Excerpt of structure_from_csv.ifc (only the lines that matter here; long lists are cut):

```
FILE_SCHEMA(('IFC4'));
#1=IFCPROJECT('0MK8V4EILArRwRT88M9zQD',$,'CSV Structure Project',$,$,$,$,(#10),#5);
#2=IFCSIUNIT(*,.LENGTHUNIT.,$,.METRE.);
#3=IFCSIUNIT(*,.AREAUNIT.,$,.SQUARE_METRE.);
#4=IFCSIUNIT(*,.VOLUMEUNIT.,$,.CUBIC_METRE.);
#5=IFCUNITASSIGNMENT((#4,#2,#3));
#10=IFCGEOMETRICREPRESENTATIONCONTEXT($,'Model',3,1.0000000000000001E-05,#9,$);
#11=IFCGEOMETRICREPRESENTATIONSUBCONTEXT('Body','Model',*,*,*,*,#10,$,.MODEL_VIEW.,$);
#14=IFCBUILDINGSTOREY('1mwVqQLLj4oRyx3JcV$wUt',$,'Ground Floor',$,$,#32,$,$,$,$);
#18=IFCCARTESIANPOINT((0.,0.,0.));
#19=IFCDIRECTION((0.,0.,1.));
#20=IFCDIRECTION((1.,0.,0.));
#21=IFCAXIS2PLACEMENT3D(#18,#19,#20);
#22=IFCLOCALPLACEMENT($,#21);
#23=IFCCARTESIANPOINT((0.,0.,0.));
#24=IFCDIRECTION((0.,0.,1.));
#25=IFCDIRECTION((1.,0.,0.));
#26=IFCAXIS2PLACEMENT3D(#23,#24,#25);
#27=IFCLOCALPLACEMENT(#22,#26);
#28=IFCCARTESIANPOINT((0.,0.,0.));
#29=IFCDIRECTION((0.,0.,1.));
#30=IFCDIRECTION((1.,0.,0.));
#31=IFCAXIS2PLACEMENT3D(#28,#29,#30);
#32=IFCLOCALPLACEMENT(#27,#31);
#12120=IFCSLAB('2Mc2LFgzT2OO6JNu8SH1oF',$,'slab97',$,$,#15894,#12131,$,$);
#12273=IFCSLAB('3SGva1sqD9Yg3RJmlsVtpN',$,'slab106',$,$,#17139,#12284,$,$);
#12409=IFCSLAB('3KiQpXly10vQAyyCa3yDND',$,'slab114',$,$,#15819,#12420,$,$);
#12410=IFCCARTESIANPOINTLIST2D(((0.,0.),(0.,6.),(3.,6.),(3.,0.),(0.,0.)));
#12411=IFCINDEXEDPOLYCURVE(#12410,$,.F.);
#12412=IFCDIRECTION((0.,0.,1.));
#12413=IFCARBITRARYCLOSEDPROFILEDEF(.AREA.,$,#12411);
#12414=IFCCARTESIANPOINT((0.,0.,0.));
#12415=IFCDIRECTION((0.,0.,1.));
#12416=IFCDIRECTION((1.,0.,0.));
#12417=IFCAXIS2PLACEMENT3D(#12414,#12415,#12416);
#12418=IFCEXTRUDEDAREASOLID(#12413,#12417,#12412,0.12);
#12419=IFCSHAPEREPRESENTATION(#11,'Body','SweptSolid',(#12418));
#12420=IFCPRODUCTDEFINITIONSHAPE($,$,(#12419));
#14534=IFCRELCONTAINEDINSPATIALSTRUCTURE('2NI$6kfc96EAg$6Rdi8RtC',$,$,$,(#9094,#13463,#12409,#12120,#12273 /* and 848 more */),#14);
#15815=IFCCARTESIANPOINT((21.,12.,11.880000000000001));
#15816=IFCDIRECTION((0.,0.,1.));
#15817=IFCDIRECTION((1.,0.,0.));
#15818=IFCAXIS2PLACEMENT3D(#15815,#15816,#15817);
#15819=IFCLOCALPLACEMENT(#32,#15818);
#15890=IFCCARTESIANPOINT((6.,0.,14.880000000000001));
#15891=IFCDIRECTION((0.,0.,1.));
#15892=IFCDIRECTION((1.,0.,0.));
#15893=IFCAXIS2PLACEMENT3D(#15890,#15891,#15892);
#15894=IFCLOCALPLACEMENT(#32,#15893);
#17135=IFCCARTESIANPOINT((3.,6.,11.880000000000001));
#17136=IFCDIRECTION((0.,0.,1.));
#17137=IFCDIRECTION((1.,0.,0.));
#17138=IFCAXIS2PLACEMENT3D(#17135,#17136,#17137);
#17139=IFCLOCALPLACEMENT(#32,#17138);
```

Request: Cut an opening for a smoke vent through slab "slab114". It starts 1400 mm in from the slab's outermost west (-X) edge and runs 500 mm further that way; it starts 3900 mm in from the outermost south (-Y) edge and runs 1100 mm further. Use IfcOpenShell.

```python
import numpy as np
import ifcopenshell
import ifcopenshell.api.feature
import ifcopenshell.api.geometry
import ifcopenshell.api.root
import ifcopenshell.geom
import ifcopenshell.util.placement
import ifcopenshell.util.representation
import ifcopenshell.util.shape
import ifcopenshell.util.unit

model = ifcopenshell.open("structure_from_csv.ifc")
unit_scale = ifcopenshell.util.unit.calculate_unit_scale(model)
settings = ifcopenshell.geom.settings()


def volume(element):
    """Net volume in cubic metres, openings subtracted."""
    shape = ifcopenshell.geom.create_shape(settings, element)
    return ifcopenshell.util.shape.get_volume(shape.geometry)


slab = model.by_id(12409)
before = volume(slab)

# Extent in the slab's own axes, in metres. The edges named are its -X and -Y sides.
slab_shape = ifcopenshell.geom.create_shape(settings, slab)
vertices = ifcopenshell.util.shape.get_vertices(slab_shape.geometry)
x_min, y_min, bottom = vertices.min(axis=0)
top = vertices[:, 2].max()

opening = ifcopenshell.api.root.create_entity(model, ifc_class="IfcOpeningElement", name="Smoke vent opening", predefined_type="OPENING")
context = ifcopenshell.util.representation.get_context(model, "Model", "Body", "MODEL_VIEW")
width, depth = 0.5, 1.1
outline = [(0.0, 0.0), (width, 0.0), (width, depth), (0.0, depth), (0.0, 0.0)]
# Overshoot both faces by 50 mm so the cut is clean.
shape = ifcopenshell.api.geometry.add_slab_representation(
    model, context=context, depth=top - bottom + 0.1, polyline=outline
)
ifcopenshell.api.geometry.assign_representation(model, product=opening, representation=shape)

matrix = ifcopenshell.util.placement.get_local_placement(slab.ObjectPlacement)
matrix[:, 3] = matrix @ np.append(np.array([x_min + 1.4, y_min + 3.9, bottom - 0.05]) / unit_scale, 1.0)
ifcopenshell.api.geometry.edit_object_placement(model, product=opening, matrix=matrix, is_si=False)
ifcopenshell.api.feature.add_feature(model, feature=opening, element=slab)

after = volume(slab)

print(f"slab volume {before:.3f} -> {after:.3f} m3")

model.write("structure_from_csv_rev.ifc")
```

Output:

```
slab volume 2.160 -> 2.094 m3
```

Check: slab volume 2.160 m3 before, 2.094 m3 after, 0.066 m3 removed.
